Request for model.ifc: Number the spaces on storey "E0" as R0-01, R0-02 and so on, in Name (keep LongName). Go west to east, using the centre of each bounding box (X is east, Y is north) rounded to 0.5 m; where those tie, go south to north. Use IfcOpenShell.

First a look at what the model holds.

```python
import ifcopenshell
import ifcopenshell.util.element
import ifcopenshell.util.placement

model = ifcopenshell.open("model.ifc")
print(model.schema)
storey = next(s for s in model.by_type("IfcBuildingStorey") if s.Name == "E0")
spaces = [e for e in ifcopenshell.util.element.get_decomposition(storey) if e.is_a("IfcSpace")]
for e in sorted(spaces, key=lambda e: e.id()):
    origin = ifcopenshell.util.placement.get_local_placement(e.ObjectPlacement)[:3, 3]
    print(e.id(), e.Name, e.LongName, origin.round(2) + 0.0, sep=" | ")
```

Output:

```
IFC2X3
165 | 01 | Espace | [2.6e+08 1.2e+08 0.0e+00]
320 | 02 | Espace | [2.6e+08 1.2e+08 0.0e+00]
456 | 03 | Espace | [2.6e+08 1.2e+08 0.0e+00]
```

```python
import ifcopenshell
import ifcopenshell.geom
import ifcopenshell.util.element
import ifcopenshell.util.shape

model = ifcopenshell.open("model.ifc")
settings = ifcopenshell.geom.settings()
settings.set("use-world-coords", True)


def centre(element):
    shape = ifcopenshell.geom.create_shape(settings, element)
    return ifcopenshell.util.shape.get_bbox_centroid(shape.geometry)


storey = next(s for s in model.by_type("IfcBuildingStorey") if s.Name == "E0")
spaces = [e for e in ifcopenshell.util.element.get_decomposition(storey) if e.is_a("IfcSpace")]

# Insertion points can sit at a corner or the storey origin, so sort by the geometry (in metres).
centres = {e: centre(e) for e in spaces}
spaces.sort(key=lambda e: (round(centres[e][0] / 0.5), centres[e][1]))

for i, e in enumerate(spaces, start=1):
    number = f"R0-{i:02d}"
    e.Name = number
    print(e.id(), number)

model.write("model_edited.ifc")
```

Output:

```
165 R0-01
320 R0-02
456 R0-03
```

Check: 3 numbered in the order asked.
